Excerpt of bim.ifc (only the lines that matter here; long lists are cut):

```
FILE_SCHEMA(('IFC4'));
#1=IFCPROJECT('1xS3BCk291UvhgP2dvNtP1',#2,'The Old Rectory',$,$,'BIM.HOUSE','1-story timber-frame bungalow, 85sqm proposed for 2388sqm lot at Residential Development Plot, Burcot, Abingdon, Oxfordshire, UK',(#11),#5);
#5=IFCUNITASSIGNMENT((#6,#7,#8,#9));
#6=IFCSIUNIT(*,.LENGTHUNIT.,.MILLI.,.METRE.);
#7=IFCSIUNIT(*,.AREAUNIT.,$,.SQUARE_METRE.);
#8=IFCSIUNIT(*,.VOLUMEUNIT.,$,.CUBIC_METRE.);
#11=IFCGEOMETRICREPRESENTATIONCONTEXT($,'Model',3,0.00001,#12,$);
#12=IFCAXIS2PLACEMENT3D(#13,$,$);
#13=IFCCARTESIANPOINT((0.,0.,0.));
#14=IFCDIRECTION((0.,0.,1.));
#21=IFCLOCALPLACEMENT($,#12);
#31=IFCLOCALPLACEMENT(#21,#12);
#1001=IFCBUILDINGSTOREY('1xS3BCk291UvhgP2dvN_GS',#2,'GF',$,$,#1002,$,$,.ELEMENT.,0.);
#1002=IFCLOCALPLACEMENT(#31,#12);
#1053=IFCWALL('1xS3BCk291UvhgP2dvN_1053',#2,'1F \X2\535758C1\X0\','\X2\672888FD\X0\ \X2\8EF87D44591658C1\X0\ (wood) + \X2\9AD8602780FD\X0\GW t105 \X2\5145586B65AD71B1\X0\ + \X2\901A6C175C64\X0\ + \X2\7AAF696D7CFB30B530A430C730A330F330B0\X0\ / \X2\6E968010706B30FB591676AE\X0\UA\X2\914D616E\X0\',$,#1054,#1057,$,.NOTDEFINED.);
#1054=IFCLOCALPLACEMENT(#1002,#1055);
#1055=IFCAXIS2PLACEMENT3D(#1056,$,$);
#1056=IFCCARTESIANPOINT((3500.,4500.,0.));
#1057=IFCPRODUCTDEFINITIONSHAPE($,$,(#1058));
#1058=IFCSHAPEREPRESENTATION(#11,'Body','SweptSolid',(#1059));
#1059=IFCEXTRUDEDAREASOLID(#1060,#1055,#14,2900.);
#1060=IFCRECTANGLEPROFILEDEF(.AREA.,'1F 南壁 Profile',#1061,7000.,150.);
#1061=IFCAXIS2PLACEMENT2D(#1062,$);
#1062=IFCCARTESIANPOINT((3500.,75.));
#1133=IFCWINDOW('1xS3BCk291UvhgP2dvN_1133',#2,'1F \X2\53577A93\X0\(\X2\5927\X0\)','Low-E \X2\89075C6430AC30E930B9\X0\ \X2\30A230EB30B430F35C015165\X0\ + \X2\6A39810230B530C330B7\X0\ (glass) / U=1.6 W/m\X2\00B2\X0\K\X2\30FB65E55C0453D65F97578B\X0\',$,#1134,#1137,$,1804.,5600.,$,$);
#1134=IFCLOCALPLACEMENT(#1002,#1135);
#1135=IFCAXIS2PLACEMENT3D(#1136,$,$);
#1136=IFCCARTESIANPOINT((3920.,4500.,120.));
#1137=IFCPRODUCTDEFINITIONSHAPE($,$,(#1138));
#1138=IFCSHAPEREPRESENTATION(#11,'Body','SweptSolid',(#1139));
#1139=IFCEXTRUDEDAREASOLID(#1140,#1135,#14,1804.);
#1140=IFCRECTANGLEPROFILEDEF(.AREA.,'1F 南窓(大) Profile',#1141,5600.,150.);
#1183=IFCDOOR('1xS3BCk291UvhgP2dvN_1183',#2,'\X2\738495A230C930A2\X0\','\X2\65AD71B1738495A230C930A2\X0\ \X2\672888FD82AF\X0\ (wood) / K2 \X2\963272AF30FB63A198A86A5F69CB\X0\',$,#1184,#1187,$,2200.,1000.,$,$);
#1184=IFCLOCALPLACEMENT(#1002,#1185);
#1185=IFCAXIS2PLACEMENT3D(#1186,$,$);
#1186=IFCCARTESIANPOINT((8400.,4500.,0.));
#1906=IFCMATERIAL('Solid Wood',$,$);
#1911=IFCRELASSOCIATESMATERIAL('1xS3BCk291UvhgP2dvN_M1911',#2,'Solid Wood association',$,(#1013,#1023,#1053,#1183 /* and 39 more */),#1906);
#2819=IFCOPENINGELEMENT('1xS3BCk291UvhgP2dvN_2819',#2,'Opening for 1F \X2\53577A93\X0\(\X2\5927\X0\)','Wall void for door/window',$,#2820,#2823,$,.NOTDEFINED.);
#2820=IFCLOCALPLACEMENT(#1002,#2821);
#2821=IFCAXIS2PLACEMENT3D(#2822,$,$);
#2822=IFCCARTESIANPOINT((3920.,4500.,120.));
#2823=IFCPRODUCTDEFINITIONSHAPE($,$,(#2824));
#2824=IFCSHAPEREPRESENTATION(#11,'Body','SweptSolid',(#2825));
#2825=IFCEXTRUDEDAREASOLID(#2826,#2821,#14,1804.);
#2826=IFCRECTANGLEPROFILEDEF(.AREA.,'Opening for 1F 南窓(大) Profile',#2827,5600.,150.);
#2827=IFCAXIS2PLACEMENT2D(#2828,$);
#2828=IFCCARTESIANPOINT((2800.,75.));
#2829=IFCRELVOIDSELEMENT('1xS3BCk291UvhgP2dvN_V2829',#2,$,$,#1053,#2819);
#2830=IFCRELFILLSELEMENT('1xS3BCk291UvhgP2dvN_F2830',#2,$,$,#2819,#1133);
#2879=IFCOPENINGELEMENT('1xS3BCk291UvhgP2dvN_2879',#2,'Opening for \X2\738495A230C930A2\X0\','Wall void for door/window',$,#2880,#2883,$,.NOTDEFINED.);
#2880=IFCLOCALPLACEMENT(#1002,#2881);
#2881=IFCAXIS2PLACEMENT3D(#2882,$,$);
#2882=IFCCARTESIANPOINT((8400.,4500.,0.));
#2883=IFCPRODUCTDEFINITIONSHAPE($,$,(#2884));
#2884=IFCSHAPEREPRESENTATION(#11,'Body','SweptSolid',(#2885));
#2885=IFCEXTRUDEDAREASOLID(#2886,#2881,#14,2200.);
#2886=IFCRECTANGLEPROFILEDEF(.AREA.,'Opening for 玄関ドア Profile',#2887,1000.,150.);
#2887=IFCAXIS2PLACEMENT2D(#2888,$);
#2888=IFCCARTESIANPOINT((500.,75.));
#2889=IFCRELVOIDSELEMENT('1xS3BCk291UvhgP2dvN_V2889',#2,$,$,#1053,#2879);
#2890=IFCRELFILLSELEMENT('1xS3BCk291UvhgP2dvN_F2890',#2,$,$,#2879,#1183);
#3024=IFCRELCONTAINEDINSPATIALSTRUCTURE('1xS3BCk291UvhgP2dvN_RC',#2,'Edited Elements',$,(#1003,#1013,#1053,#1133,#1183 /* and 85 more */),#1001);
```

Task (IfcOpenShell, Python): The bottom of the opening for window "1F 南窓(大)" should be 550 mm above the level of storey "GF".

```python
import numpy as np
import ifcopenshell
import ifcopenshell.api.geometry
import ifcopenshell.geom
import ifcopenshell.util.element
import ifcopenshell.util.placement
import ifcopenshell.util.shape
import ifcopenshell.util.unit

model = ifcopenshell.open("bim.ifc")
unit_scale = ifcopenshell.util.unit.calculate_unit_scale(model)

window = model.by_guid("1xS3BCk291UvhgP2dvN_1133")
opening = window.FillsVoids[0].RelatingOpeningElement
storey = ifcopenshell.util.element.get_container(window, ifc_class="IfcBuildingStorey")
level = ifcopenshell.util.placement.get_local_placement(storey.ObjectPlacement)[2, 3]

# The opening's origin need not be at the sill, so measure its lowest point.
shape = ifcopenshell.geom.create_shape(ifcopenshell.geom.settings(), opening)
bottom = ifcopenshell.util.shape.get_shape_bottom_elevation(shape, shape.geometry) / unit_scale
dz = level + 0.55 / unit_scale - bottom

shift = np.array([0.0, 0.0, dz])
# The window is not placed relative to its opening, so move both.
for product in (opening, window):
    matrix = ifcopenshell.util.placement.get_local_placement(product.ObjectPlacement)
    matrix[:3, 3] += shift
    ifcopenshell.api.geometry.edit_object_placement(model, product=product, matrix=matrix, is_si=False)

print(f"moved by {dz * unit_scale:+.3f} m")

model.write("bim_updated.ifc")
```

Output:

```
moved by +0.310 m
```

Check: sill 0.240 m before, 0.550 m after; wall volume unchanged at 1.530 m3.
